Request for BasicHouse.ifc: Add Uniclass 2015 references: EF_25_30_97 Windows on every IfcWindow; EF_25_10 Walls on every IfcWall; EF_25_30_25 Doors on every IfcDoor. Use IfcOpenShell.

First a look at what the model holds.

```python
import ifcopenshell

model = ifcopenshell.open("BasicHouse.ifc")
print(model.schema)
print("classifications:", [c.Name for c in model.by_type("IfcClassification")])
for ifc_class in ("IfcDoor", "IfcRoof", "IfcStair", "IfcWall", "IfcWindow"):
    print(ifc_class, len(model.by_type(ifc_class)))
```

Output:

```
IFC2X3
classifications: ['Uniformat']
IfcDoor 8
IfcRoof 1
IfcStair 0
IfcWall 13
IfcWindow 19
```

```python
import ifcopenshell
import ifcopenshell.api.classification

model = ifcopenshell.open("BasicHouse.ifc")

# IFC2X3 requires Source and Edition and has no link from the project to the system.
system = model.create_entity("IfcClassification", Source="NBS", Edition="2015", Name="Uniclass 2015")

codes = {
    "IfcWindow": ("EF_25_30_97", "Windows"),
    "IfcWall": ("EF_25_10", "Walls"),
    "IfcDoor": ("EF_25_30_25", "Doors"),
}
for ifc_class, (code, name) in codes.items():
    products = model.by_type(ifc_class)
    ifcopenshell.api.classification.add_reference(
        model, products=products, classification=system, identification=code, name=name
    )
    print(code, len(products))

model.write("BasicHouse_rev.ifc")
```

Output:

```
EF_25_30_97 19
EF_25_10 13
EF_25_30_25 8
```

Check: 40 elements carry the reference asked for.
